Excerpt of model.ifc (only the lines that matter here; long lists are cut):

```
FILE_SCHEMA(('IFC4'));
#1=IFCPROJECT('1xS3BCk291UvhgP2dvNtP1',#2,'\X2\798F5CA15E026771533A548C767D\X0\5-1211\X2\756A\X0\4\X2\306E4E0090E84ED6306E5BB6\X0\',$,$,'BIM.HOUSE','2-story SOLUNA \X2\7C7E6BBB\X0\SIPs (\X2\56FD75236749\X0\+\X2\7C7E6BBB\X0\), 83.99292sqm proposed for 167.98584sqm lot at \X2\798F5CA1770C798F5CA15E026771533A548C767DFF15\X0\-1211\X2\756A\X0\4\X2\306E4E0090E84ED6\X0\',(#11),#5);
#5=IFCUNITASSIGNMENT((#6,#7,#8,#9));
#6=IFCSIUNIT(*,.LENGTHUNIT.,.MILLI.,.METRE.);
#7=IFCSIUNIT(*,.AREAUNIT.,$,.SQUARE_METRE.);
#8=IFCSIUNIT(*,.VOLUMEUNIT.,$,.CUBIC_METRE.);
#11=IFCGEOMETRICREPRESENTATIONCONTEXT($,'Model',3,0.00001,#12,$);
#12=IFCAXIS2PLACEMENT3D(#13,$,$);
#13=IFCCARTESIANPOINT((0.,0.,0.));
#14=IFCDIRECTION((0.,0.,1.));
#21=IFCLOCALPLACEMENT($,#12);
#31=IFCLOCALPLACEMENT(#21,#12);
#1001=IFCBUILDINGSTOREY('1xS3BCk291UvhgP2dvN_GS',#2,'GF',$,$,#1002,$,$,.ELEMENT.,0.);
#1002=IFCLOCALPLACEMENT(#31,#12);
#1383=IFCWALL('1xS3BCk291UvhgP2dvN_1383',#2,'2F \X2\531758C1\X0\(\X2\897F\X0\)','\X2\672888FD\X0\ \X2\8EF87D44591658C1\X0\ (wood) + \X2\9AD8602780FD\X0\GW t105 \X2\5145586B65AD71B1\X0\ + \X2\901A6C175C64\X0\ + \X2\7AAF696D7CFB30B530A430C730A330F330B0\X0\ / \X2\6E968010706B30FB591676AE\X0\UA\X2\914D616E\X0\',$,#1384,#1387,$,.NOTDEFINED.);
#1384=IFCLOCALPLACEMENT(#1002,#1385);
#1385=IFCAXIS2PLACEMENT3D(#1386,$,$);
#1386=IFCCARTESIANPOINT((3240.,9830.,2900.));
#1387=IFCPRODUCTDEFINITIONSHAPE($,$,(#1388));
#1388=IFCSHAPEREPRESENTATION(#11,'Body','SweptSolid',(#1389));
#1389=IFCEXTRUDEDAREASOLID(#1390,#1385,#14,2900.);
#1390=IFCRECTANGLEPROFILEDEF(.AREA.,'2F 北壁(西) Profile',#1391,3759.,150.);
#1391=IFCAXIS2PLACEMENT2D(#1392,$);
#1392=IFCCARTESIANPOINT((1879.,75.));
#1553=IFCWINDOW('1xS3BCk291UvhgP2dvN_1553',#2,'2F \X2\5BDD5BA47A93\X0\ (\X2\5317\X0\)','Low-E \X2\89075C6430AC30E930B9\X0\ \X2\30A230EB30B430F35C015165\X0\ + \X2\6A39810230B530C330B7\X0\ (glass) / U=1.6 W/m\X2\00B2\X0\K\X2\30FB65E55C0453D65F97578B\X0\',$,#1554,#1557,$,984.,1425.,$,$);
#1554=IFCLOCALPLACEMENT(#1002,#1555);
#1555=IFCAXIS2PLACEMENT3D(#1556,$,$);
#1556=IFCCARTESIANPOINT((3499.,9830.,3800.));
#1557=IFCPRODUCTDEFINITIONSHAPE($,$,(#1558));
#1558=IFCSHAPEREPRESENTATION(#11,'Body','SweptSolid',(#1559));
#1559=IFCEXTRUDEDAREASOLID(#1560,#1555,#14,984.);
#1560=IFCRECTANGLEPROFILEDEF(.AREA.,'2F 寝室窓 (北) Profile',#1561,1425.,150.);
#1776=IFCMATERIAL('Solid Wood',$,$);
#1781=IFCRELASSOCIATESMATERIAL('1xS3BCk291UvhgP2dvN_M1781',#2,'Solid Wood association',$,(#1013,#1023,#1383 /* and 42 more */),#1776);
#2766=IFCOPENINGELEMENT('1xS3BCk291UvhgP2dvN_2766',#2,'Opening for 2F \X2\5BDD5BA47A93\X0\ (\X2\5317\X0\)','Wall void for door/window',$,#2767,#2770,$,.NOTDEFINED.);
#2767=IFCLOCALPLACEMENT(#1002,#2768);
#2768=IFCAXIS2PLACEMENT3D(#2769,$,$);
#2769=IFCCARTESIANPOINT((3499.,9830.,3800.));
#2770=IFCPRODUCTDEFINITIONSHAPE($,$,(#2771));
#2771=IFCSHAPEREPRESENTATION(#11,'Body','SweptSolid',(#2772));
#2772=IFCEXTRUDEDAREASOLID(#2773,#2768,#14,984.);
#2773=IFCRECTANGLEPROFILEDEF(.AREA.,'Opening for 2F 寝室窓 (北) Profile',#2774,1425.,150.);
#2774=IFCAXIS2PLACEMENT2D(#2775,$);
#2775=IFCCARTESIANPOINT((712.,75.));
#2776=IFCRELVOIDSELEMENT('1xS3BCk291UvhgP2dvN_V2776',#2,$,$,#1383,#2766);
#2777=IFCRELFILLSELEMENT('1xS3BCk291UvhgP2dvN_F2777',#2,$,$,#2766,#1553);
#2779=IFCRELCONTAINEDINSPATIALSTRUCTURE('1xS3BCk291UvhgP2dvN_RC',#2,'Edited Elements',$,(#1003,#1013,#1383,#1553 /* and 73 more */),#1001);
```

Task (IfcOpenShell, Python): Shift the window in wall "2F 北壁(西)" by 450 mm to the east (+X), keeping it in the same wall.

```python
import ifcopenshell
import ifcopenshell.api.geometry
import ifcopenshell.util.placement

model = ifcopenshell.open("model.ifc")

window = model.by_id(1553)
opening = window.FillsVoids[0].RelatingOpeningElement
wall = opening.VoidsElements[0].RelatingBuildingElement

wall_matrix = ifcopenshell.util.placement.get_local_placement(wall.ObjectPlacement)
shift = wall_matrix[:3, 0] * 450.0
before = ifcopenshell.util.placement.get_local_placement(window.ObjectPlacement)[:3, 3].copy()

# The window is not placed relative to its opening, so move both.
for product in (opening, window):
    matrix = ifcopenshell.util.placement.get_local_placement(product.ObjectPlacement)
    matrix[:3, 3] += shift
    ifcopenshell.api.geometry.edit_object_placement(model, product=product, matrix=matrix, is_si=False)

after = ifcopenshell.util.placement.get_local_placement(window.ObjectPlacement)[:3, 3]
print("window moved by", (after - before).round(3) + 0.0)

model.write("model-out.ifc")
```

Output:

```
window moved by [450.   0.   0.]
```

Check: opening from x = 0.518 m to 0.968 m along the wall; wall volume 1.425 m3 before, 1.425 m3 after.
